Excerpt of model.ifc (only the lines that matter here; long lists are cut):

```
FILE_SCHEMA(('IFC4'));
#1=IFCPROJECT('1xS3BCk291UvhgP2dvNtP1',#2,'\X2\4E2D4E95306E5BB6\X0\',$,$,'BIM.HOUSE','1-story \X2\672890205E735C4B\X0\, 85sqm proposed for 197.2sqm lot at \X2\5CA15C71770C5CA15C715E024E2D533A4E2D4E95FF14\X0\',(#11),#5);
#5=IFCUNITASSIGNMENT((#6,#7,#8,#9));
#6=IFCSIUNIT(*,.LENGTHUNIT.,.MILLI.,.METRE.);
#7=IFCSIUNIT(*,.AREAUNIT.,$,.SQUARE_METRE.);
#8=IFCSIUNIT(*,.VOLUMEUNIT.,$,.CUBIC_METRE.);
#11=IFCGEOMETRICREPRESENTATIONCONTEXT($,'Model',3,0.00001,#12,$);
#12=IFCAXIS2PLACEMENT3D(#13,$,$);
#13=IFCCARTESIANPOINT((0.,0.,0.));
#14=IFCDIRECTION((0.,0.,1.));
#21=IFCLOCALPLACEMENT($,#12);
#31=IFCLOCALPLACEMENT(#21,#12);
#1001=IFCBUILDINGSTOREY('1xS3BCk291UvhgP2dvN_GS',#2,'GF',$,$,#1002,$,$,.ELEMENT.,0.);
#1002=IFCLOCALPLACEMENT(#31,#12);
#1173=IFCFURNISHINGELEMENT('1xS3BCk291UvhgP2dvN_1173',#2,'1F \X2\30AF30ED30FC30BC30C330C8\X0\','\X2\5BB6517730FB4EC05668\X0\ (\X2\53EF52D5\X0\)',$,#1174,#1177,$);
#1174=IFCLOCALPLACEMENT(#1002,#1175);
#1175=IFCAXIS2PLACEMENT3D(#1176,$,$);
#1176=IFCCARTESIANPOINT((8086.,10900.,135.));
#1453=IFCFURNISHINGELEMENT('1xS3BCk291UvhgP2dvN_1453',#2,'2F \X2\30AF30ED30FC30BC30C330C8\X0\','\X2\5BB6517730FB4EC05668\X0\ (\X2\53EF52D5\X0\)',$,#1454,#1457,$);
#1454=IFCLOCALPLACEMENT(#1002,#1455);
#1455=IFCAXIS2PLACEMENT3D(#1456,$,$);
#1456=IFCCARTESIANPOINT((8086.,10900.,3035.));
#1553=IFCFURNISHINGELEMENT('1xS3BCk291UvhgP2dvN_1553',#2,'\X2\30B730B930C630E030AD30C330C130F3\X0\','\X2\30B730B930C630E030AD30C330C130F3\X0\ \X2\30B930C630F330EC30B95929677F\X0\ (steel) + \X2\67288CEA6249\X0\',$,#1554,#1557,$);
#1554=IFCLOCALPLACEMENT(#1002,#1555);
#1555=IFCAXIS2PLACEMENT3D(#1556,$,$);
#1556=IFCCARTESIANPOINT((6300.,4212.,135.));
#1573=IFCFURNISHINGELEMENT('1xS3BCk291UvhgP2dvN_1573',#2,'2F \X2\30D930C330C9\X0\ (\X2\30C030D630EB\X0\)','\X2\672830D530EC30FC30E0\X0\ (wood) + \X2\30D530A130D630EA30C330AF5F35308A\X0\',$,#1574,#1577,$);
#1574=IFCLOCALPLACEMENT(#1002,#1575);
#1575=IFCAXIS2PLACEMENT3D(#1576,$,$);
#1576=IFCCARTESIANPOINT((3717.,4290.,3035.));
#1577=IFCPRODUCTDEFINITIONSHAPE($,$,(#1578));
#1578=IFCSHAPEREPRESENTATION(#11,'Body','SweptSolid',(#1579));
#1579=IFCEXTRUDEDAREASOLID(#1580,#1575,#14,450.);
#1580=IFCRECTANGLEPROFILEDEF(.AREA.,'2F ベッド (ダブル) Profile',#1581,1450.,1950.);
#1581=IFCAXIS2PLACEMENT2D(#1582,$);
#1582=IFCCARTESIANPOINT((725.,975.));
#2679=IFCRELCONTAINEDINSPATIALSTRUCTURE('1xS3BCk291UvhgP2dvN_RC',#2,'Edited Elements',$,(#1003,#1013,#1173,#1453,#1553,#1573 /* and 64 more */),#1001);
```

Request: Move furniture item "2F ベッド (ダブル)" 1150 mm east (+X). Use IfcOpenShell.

```python
import ifcopenshell
import ifcopenshell.api.geometry
import ifcopenshell.util.placement
import ifcopenshell.util.unit

model = ifcopenshell.open("model.ifc")
unit_scale = ifcopenshell.util.unit.calculate_unit_scale(model)

item = model.by_id(1573)
matrix = ifcopenshell.util.placement.get_local_placement(item.ObjectPlacement)
matrix[0, 3] += 1.15 / unit_scale
ifcopenshell.api.geometry.edit_object_placement(model, product=item, matrix=matrix, is_si=False)

print(ifcopenshell.util.placement.get_local_placement(item.ObjectPlacement).round(3) + 0.0)

model.write("model_rev.ifc")
```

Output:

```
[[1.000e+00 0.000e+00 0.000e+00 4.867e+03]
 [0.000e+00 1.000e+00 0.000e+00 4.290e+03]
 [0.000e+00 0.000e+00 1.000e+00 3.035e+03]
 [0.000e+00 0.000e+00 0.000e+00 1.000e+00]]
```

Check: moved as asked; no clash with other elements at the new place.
